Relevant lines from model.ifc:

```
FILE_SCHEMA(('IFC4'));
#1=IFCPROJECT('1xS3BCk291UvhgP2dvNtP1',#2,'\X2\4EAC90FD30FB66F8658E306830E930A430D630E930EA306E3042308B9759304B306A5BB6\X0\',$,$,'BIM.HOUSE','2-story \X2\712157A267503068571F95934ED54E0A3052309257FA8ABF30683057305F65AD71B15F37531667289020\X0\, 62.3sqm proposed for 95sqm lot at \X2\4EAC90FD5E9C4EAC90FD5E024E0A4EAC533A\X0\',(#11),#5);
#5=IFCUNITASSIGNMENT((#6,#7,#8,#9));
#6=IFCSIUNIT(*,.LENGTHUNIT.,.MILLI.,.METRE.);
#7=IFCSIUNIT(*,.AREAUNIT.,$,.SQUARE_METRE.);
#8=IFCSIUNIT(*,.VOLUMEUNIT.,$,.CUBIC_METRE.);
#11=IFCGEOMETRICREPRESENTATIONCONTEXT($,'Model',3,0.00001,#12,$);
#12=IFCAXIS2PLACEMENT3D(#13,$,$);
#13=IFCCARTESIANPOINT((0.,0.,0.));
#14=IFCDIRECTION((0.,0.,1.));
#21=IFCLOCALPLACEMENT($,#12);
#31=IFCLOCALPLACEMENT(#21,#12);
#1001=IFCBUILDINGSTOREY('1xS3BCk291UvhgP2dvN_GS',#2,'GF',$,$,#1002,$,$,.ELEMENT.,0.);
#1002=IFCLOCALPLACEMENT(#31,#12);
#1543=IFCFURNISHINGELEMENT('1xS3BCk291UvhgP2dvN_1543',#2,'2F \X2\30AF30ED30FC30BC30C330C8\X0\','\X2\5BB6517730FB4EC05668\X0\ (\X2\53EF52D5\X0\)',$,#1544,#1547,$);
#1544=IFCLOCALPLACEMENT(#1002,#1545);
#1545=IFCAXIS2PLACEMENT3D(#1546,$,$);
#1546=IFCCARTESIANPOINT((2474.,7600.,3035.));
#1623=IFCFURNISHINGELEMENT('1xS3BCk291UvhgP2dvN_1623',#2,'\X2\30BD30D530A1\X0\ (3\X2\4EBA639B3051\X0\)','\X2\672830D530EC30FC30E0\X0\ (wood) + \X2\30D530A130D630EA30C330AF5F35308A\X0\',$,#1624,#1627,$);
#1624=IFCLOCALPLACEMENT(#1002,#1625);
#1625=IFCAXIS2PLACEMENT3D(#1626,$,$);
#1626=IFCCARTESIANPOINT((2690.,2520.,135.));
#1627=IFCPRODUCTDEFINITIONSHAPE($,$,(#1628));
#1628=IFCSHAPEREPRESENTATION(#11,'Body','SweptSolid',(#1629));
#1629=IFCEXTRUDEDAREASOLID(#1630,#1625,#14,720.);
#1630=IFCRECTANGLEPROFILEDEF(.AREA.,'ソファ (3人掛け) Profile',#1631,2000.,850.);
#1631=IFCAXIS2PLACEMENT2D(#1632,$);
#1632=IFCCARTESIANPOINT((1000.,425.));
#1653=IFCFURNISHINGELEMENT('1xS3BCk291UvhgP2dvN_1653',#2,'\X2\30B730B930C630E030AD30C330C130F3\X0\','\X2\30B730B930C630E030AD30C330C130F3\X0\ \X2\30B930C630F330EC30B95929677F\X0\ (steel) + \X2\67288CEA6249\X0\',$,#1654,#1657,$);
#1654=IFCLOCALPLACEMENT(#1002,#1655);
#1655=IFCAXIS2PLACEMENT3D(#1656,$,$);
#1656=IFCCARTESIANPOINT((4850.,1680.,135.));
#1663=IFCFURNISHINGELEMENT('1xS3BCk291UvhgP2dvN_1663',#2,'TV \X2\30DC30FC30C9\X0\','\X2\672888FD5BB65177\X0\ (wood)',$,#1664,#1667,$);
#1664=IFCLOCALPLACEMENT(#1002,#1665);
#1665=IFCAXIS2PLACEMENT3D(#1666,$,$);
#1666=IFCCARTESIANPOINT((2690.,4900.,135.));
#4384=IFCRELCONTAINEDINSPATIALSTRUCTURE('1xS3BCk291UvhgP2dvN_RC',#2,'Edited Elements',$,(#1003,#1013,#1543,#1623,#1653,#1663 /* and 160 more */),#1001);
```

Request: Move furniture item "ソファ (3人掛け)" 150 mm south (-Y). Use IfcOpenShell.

```python
import ifcopenshell
import ifcopenshell.api.geometry
import ifcopenshell.util.placement
import ifcopenshell.util.unit

model = ifcopenshell.open("model.ifc")
unit_scale = ifcopenshell.util.unit.calculate_unit_scale(model)

item = model.by_guid("1xS3BCk291UvhgP2dvN_1623")
matrix = ifcopenshell.util.placement.get_local_placement(item.ObjectPlacement)
matrix[1, 3] -= 0.15 / unit_scale
ifcopenshell.api.geometry.edit_object_placement(model, product=item, matrix=matrix, is_si=False)

print(ifcopenshell.util.placement.get_local_placement(item.ObjectPlacement).round(3) + 0.0)

model.write("model_edited.ifc")
```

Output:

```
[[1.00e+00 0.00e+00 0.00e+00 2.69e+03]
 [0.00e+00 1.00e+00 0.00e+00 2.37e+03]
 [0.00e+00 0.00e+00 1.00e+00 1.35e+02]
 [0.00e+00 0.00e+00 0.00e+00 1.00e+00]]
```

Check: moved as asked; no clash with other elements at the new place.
